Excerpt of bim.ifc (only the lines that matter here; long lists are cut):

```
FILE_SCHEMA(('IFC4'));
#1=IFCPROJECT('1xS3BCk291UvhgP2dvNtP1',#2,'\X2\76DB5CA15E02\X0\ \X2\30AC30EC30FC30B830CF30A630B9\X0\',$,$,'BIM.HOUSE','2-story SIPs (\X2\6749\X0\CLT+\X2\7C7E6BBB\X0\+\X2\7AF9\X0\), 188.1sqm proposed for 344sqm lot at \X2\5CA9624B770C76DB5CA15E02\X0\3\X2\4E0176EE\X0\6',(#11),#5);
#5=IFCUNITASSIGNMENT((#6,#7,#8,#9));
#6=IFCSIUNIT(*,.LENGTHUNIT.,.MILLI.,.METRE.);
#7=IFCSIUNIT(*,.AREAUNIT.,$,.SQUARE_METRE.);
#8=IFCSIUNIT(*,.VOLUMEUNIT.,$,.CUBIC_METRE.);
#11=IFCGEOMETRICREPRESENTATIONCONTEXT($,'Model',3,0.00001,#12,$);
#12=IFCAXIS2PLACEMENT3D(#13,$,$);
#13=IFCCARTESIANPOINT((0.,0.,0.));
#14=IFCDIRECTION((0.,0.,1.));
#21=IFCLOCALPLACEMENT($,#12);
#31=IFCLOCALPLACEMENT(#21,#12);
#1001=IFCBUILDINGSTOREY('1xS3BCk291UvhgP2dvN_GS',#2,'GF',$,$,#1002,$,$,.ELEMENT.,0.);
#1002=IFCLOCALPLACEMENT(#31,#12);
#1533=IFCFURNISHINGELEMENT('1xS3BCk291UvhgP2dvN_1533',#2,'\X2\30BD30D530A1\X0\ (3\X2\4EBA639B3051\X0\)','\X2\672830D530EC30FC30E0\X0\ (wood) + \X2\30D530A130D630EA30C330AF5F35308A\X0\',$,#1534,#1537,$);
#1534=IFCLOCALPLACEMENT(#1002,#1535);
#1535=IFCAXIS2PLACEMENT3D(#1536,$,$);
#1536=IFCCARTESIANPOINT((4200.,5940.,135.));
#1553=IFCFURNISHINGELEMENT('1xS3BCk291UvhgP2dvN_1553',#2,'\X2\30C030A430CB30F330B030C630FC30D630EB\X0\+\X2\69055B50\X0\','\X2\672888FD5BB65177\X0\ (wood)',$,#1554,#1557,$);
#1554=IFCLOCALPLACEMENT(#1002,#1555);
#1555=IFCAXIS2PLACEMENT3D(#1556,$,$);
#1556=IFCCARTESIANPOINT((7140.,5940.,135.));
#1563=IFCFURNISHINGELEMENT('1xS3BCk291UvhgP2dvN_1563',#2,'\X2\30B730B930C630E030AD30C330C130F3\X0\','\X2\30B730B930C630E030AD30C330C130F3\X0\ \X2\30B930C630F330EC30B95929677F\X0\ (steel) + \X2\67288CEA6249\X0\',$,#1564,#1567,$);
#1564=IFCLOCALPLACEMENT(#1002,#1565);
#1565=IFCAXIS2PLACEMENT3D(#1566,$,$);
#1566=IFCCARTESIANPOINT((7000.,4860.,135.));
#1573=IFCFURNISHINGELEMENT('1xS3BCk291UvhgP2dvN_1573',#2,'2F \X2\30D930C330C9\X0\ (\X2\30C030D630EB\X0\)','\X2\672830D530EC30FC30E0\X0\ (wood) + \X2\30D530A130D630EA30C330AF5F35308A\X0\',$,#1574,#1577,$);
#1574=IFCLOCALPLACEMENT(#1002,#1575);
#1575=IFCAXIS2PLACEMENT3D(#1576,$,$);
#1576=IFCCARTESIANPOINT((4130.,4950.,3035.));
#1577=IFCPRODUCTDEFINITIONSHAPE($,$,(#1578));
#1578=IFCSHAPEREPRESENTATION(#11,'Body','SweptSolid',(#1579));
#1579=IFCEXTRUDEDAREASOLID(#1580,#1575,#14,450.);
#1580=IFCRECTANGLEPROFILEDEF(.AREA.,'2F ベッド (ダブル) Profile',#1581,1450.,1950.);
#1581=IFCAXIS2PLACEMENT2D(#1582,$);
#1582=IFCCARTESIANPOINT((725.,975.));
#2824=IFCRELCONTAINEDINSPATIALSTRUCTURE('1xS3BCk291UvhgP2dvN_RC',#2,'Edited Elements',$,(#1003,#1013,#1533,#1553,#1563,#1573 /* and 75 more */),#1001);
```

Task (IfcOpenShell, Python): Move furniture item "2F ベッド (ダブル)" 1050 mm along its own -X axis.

```python
import ifcopenshell
import ifcopenshell.api.geometry
import ifcopenshell.util.placement
import ifcopenshell.util.unit

model = ifcopenshell.open("bim.ifc")
unit_scale = ifcopenshell.util.unit.calculate_unit_scale(model)

item = model.by_guid("1xS3BCk291UvhgP2dvN_1573")
matrix = ifcopenshell.util.placement.get_local_placement(item.ObjectPlacement)
matrix[:3, 3] -= matrix[:3, 0] * 1.05 / unit_scale
ifcopenshell.api.geometry.edit_object_placement(model, product=item, matrix=matrix, is_si=False)

print(ifcopenshell.util.placement.get_local_placement(item.ObjectPlacement).round(3) + 0.0)

model.write("bim_edited.ifc")
```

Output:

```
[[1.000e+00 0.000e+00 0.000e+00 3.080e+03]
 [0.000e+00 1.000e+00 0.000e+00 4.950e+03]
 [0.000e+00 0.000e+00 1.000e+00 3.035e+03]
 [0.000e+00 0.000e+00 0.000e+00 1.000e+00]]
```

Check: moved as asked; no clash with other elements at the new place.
